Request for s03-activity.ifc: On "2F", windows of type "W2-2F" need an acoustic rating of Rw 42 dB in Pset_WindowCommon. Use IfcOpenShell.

First a look at what the model holds.

```python
import ifcopenshell
import ifcopenshell.util.element

model = ifcopenshell.open("s03-activity.ifc")
print(model.schema)
storey = next(s for s in model.by_type("IfcBuildingStorey") if s.Name == "2F")
windows = [e for e in ifcopenshell.util.element.get_decomposition(storey) if e.is_a("IfcWindow")]
seen = {}
for e in windows:
    element_type = ifcopenshell.util.element.get_type(e)
    key = (element_type.Name if element_type != e and element_type else None, ifcopenshell.util.element.get_pset(e, "Pset_WindowCommon", "AcousticRating"))
    seen[key] = seen.get(key, 0) + 1
for (name, value), count in sorted(seen.items(), key=str):
    print(count, "x", name, "|", value)
```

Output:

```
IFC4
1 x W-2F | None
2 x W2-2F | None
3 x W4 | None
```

```python
import ifcopenshell
import ifcopenshell.api.pset
import ifcopenshell.util.element

model = ifcopenshell.open("s03-activity.ifc")

storey = next(s for s in model.by_type("IfcBuildingStorey") if s.Name == "2F")
windows = [e for e in ifcopenshell.util.element.get_decomposition(storey) if e.is_a("IfcWindow")]

count = 0
for e in windows:
    element_type = ifcopenshell.util.element.get_type(e)
    if element_type in (None, e) or element_type.Name != "W2-2F":
        continue
    # add_pset returns the element's existing set when there is one.
    pset = ifcopenshell.api.pset.add_pset(model, product=e, name="Pset_WindowCommon")
    ifcopenshell.api.pset.edit_pset(model, pset=pset, properties={"AcousticRating": "Rw 42 dB"})
    count += 1

print(count, "windows updated")

model.write("s03-activity-out.ifc")
```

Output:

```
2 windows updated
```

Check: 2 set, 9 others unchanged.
